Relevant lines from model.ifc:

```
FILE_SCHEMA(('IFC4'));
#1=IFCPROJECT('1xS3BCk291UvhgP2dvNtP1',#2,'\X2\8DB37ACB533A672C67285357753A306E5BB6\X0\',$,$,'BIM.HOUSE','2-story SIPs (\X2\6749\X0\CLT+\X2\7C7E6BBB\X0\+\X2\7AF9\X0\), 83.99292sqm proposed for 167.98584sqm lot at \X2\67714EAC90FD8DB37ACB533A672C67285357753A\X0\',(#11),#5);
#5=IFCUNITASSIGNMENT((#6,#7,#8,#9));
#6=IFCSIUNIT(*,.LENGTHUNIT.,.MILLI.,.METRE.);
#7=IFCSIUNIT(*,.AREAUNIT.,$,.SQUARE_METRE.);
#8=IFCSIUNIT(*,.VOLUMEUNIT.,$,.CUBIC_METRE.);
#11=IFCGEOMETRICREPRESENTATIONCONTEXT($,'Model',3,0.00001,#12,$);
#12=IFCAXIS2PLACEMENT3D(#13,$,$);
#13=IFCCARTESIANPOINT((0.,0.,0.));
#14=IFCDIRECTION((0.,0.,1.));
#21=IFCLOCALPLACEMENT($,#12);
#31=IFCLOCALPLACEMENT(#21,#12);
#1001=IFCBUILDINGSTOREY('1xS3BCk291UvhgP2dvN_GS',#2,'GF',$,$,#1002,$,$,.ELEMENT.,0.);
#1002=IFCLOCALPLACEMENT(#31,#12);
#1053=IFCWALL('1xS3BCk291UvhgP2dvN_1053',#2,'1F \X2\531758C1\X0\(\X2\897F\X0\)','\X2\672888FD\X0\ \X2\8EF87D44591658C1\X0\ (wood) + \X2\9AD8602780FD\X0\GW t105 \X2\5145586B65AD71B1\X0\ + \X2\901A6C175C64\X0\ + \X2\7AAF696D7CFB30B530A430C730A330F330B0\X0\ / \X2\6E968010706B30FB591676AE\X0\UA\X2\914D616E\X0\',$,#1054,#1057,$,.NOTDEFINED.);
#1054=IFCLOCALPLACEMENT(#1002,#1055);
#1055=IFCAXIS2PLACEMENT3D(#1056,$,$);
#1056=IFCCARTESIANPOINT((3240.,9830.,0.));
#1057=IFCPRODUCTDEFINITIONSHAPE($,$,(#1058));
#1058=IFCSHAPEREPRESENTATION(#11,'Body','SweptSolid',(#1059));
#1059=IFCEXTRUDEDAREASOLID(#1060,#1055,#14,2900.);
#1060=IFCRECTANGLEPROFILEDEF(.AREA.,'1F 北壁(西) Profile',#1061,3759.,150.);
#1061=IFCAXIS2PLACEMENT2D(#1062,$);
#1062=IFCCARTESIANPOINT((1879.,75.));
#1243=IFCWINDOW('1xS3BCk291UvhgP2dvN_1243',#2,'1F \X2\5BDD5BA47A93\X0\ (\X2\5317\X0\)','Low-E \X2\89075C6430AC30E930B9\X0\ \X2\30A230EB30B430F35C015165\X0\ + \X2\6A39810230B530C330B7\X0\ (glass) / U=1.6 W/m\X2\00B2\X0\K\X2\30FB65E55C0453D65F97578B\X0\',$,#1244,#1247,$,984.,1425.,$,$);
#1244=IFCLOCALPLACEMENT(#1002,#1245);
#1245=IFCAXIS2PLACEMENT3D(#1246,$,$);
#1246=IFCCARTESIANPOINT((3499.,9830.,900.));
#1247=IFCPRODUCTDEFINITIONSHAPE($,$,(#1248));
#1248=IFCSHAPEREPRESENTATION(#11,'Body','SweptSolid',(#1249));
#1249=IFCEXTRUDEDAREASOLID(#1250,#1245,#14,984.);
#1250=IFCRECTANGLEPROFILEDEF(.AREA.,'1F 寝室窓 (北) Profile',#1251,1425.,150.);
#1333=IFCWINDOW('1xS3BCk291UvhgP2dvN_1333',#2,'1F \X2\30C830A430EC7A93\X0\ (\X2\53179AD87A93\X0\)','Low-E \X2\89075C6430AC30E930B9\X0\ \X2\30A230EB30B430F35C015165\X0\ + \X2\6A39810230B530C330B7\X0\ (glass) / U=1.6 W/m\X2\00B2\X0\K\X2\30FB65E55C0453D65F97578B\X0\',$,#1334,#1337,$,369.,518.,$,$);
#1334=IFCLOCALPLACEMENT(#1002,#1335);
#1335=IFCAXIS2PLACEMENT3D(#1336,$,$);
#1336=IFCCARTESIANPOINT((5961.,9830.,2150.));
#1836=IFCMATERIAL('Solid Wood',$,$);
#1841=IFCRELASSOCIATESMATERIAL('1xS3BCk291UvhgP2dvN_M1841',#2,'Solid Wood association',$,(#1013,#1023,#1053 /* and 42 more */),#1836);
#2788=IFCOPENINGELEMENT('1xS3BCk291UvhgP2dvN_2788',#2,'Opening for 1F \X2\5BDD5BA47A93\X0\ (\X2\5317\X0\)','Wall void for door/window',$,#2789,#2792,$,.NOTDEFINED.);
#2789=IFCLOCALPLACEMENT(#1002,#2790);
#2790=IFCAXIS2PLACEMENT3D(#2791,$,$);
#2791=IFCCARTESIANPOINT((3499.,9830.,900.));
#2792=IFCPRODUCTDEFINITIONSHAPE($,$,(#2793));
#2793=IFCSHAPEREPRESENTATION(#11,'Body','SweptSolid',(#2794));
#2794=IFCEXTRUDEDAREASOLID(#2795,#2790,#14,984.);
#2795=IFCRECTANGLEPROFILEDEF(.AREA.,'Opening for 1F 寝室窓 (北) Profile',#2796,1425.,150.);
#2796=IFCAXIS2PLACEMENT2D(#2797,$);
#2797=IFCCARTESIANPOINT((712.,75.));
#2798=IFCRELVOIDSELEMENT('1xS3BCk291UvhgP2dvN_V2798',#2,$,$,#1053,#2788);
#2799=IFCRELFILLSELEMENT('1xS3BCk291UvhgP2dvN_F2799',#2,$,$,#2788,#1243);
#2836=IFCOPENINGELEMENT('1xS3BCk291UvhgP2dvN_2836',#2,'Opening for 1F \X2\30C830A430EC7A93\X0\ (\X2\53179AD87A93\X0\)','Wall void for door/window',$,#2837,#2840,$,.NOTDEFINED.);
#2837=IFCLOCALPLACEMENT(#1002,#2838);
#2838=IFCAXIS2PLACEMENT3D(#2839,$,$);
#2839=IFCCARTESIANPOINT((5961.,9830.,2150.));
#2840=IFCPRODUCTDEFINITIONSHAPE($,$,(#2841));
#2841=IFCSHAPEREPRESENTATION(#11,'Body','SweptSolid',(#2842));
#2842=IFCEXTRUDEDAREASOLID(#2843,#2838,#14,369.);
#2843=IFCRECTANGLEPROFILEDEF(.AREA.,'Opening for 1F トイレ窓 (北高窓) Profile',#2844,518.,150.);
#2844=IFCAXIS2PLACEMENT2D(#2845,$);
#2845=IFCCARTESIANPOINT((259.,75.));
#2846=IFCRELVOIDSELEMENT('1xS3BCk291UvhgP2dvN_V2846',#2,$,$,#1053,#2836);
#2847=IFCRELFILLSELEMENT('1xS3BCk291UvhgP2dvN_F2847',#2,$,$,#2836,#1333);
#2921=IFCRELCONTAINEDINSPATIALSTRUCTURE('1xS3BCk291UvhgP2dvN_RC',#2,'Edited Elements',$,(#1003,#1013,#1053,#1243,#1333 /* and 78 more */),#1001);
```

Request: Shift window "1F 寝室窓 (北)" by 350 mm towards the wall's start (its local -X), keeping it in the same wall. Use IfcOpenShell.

```python
import ifcopenshell
import ifcopenshell.api.geometry
import ifcopenshell.util.placement

model = ifcopenshell.open("model.ifc")

window = model.by_guid("1xS3BCk291UvhgP2dvN_1243")
opening = window.FillsVoids[0].RelatingOpeningElement
wall = opening.VoidsElements[0].RelatingBuildingElement

wall_matrix = ifcopenshell.util.placement.get_local_placement(wall.ObjectPlacement)
shift = wall_matrix[:3, 0] * -350.0
before = ifcopenshell.util.placement.get_local_placement(window.ObjectPlacement)[:3, 3].copy()

# The window is not placed relative to its opening, so move both.
for product in (opening, window):
    matrix = ifcopenshell.util.placement.get_local_placement(product.ObjectPlacement)
    matrix[:3, 3] += shift
    ifcopenshell.api.geometry.edit_object_placement(model, product=product, matrix=matrix, is_si=False)

after = ifcopenshell.util.placement.get_local_placement(window.ObjectPlacement)[:3, 3]
print("window moved by", (after - before).round(3) + 0.0)

model.write("model_v2.ifc")
```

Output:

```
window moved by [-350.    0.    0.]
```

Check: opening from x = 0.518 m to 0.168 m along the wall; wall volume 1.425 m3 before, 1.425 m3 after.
